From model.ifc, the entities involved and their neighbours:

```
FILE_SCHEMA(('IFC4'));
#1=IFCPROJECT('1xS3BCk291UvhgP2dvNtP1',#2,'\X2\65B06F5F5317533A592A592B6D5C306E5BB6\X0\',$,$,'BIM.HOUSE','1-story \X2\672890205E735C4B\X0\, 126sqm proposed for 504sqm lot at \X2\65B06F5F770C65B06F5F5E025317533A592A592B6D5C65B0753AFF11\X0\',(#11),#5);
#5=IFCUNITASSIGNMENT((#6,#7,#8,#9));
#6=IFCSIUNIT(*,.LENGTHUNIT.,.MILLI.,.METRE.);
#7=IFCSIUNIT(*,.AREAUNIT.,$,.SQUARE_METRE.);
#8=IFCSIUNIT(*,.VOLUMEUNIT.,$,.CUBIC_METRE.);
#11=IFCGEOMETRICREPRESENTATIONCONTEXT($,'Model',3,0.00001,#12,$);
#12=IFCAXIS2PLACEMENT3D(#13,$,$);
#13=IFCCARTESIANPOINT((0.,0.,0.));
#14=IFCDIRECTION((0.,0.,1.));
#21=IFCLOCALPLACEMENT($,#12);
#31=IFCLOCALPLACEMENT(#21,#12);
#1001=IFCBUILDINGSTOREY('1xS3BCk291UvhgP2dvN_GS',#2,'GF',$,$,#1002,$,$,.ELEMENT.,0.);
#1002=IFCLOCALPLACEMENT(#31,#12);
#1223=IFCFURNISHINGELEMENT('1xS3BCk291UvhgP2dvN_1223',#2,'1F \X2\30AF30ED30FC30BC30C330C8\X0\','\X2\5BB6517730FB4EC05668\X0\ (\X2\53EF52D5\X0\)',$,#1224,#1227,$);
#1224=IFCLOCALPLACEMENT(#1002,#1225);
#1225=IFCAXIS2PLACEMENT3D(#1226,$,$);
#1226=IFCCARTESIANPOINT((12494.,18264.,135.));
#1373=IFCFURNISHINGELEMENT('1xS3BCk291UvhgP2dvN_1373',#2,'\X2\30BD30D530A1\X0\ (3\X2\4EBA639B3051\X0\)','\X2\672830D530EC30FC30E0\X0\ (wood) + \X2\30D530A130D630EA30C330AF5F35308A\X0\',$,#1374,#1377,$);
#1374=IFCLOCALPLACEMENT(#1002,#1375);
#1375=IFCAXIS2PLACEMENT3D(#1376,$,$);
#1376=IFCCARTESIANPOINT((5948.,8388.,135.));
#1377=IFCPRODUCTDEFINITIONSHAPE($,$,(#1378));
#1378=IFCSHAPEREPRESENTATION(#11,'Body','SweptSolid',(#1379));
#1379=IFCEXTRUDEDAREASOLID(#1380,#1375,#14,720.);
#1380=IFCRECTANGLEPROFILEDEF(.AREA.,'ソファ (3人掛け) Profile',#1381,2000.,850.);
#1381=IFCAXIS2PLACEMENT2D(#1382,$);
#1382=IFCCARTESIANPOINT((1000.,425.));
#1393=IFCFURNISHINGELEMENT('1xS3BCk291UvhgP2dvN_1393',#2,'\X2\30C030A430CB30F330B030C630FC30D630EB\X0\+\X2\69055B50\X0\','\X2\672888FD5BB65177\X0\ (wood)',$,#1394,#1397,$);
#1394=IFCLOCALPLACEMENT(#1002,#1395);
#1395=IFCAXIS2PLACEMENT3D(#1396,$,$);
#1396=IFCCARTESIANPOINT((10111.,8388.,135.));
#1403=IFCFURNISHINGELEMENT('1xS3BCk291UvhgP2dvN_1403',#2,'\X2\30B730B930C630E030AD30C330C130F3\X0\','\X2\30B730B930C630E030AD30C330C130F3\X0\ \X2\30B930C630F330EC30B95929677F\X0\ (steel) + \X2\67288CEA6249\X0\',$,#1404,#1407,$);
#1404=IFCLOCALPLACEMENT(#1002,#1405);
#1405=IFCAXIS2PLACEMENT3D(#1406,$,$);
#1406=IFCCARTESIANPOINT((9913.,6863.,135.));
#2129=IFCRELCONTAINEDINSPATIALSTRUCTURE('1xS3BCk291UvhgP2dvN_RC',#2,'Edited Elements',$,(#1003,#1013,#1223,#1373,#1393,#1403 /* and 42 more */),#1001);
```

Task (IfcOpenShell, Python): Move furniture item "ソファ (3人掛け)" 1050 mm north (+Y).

```python
import ifcopenshell
import ifcopenshell.api.geometry
import ifcopenshell.util.placement

model = ifcopenshell.open("model.ifc")

item = model.by_guid("1xS3BCk291UvhgP2dvN_1373")
matrix = ifcopenshell.util.placement.get_local_placement(item.ObjectPlacement)
matrix[1, 3] += 1050.0
ifcopenshell.api.geometry.edit_object_placement(model, product=item, matrix=matrix, is_si=False)

print(ifcopenshell.util.placement.get_local_placement(item.ObjectPlacement).round(3) + 0.0)

model.write("model_updated.ifc")
```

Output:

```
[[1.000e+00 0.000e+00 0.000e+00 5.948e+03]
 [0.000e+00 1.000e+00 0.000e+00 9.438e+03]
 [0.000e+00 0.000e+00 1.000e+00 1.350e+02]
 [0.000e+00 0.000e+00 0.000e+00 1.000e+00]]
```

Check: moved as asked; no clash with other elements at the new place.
